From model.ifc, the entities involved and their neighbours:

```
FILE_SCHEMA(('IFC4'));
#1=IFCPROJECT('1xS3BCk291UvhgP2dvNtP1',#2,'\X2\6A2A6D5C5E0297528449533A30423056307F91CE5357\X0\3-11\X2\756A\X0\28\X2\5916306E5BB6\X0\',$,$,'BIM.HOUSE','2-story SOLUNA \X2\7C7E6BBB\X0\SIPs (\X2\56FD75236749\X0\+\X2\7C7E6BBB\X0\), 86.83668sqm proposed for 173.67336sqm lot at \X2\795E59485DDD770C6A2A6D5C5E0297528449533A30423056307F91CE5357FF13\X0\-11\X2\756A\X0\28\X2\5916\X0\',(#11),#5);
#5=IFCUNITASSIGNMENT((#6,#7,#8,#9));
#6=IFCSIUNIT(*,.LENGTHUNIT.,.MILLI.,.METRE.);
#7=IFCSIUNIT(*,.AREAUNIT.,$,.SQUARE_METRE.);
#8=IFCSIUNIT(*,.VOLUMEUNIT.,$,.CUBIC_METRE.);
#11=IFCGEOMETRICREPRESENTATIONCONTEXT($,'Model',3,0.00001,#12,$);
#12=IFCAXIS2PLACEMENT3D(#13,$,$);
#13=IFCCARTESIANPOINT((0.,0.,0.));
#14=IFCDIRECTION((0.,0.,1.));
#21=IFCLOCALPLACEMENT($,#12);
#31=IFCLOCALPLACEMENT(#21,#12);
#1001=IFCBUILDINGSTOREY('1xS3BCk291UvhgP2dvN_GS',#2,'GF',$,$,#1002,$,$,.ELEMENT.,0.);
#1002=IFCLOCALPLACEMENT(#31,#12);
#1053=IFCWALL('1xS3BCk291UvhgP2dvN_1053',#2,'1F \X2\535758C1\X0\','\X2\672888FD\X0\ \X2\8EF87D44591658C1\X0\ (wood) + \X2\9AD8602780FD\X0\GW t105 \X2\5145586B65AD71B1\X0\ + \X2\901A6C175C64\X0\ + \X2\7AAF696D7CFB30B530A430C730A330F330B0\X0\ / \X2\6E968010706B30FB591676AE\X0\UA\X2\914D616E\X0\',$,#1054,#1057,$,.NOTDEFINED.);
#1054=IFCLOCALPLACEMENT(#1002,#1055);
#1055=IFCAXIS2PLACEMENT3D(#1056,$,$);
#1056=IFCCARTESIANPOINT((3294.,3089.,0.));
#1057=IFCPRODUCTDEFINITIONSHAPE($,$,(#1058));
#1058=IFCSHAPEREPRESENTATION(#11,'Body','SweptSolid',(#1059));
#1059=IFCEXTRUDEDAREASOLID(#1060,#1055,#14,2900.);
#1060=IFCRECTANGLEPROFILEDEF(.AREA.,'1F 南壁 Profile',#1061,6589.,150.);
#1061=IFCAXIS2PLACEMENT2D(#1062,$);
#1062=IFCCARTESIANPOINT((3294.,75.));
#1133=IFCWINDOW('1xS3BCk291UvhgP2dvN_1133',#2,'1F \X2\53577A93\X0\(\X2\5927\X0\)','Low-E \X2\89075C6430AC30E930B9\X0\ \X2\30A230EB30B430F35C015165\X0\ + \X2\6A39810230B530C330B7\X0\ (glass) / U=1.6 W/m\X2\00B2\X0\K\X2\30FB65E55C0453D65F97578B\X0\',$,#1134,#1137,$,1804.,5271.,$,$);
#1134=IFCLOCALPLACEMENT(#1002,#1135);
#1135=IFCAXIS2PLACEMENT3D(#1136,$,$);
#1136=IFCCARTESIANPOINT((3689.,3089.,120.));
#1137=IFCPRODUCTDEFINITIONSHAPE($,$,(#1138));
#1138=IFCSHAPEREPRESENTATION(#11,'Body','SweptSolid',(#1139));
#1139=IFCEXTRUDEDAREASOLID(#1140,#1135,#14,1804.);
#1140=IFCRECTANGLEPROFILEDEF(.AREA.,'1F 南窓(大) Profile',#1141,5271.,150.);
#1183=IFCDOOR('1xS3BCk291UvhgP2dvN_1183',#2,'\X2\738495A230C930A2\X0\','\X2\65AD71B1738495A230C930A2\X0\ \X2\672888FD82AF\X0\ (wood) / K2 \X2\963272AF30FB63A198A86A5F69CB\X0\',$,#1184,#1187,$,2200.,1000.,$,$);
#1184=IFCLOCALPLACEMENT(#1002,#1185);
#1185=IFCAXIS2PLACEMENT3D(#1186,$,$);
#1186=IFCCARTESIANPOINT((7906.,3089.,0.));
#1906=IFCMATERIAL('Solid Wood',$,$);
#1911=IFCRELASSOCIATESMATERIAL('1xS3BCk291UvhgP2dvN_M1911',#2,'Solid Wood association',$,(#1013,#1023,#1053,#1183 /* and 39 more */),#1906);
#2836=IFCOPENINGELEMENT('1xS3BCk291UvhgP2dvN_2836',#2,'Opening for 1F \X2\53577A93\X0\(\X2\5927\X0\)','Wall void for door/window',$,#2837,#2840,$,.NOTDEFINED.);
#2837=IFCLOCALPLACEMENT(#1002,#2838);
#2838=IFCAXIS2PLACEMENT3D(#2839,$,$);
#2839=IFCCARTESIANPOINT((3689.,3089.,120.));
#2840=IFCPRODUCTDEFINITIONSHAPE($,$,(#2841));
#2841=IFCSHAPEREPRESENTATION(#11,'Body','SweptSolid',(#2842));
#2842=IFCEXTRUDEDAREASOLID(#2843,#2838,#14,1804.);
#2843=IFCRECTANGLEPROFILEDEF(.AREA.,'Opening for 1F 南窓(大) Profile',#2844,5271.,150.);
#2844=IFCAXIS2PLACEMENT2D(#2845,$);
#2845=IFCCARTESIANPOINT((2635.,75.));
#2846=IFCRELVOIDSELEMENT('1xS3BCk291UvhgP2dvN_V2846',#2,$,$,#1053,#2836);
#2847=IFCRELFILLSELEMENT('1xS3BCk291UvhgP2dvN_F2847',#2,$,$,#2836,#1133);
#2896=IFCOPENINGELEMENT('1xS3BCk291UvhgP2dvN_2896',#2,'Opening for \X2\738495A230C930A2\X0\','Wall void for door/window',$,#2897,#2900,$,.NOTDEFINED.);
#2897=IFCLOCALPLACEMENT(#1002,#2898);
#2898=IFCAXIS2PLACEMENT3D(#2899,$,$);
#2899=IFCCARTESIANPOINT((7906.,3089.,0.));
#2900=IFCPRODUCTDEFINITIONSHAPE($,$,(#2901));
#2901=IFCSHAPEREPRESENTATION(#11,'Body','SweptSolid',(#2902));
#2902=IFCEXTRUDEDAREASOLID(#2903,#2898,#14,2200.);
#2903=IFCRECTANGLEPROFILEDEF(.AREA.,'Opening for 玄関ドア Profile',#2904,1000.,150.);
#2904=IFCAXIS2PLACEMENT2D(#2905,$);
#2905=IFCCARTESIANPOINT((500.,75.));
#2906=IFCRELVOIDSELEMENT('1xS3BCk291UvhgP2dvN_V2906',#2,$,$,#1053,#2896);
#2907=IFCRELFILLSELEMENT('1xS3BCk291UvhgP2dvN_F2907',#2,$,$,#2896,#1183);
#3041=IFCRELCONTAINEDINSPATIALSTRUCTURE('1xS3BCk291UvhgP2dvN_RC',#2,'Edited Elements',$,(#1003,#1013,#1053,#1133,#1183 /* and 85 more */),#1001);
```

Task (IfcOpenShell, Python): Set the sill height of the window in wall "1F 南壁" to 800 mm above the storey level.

```python
import numpy as np
import ifcopenshell
import ifcopenshell.api.geometry
import ifcopenshell.geom
import ifcopenshell.util.element
import ifcopenshell.util.placement
import ifcopenshell.util.shape
import ifcopenshell.util.unit

model = ifcopenshell.open("model.ifc")
unit_scale = ifcopenshell.util.unit.calculate_unit_scale(model)

window = model.by_id(1133)
opening = window.FillsVoids[0].RelatingOpeningElement
storey = ifcopenshell.util.element.get_container(window, ifc_class="IfcBuildingStorey")
level = ifcopenshell.util.placement.get_local_placement(storey.ObjectPlacement)[2, 3]

# The opening's origin need not be at the sill, so measure its lowest point.
shape = ifcopenshell.geom.create_shape(ifcopenshell.geom.settings(), opening)
bottom = ifcopenshell.util.shape.get_shape_bottom_elevation(shape, shape.geometry) / unit_scale
dz = level + 800.0 - bottom

shift = np.array([0.0, 0.0, dz])
# The window is not placed relative to its opening, so move both.
for product in (opening, window):
    matrix = ifcopenshell.util.placement.get_local_placement(product.ObjectPlacement)
    matrix[:3, 3] += shift
    ifcopenshell.api.geometry.edit_object_placement(model, product=product, matrix=matrix, is_si=False)

print(f"moved by {dz * unit_scale:+.3f} m")

model.write("model_v2.ifc")
```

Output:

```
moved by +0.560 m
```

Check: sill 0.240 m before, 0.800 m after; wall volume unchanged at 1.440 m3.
